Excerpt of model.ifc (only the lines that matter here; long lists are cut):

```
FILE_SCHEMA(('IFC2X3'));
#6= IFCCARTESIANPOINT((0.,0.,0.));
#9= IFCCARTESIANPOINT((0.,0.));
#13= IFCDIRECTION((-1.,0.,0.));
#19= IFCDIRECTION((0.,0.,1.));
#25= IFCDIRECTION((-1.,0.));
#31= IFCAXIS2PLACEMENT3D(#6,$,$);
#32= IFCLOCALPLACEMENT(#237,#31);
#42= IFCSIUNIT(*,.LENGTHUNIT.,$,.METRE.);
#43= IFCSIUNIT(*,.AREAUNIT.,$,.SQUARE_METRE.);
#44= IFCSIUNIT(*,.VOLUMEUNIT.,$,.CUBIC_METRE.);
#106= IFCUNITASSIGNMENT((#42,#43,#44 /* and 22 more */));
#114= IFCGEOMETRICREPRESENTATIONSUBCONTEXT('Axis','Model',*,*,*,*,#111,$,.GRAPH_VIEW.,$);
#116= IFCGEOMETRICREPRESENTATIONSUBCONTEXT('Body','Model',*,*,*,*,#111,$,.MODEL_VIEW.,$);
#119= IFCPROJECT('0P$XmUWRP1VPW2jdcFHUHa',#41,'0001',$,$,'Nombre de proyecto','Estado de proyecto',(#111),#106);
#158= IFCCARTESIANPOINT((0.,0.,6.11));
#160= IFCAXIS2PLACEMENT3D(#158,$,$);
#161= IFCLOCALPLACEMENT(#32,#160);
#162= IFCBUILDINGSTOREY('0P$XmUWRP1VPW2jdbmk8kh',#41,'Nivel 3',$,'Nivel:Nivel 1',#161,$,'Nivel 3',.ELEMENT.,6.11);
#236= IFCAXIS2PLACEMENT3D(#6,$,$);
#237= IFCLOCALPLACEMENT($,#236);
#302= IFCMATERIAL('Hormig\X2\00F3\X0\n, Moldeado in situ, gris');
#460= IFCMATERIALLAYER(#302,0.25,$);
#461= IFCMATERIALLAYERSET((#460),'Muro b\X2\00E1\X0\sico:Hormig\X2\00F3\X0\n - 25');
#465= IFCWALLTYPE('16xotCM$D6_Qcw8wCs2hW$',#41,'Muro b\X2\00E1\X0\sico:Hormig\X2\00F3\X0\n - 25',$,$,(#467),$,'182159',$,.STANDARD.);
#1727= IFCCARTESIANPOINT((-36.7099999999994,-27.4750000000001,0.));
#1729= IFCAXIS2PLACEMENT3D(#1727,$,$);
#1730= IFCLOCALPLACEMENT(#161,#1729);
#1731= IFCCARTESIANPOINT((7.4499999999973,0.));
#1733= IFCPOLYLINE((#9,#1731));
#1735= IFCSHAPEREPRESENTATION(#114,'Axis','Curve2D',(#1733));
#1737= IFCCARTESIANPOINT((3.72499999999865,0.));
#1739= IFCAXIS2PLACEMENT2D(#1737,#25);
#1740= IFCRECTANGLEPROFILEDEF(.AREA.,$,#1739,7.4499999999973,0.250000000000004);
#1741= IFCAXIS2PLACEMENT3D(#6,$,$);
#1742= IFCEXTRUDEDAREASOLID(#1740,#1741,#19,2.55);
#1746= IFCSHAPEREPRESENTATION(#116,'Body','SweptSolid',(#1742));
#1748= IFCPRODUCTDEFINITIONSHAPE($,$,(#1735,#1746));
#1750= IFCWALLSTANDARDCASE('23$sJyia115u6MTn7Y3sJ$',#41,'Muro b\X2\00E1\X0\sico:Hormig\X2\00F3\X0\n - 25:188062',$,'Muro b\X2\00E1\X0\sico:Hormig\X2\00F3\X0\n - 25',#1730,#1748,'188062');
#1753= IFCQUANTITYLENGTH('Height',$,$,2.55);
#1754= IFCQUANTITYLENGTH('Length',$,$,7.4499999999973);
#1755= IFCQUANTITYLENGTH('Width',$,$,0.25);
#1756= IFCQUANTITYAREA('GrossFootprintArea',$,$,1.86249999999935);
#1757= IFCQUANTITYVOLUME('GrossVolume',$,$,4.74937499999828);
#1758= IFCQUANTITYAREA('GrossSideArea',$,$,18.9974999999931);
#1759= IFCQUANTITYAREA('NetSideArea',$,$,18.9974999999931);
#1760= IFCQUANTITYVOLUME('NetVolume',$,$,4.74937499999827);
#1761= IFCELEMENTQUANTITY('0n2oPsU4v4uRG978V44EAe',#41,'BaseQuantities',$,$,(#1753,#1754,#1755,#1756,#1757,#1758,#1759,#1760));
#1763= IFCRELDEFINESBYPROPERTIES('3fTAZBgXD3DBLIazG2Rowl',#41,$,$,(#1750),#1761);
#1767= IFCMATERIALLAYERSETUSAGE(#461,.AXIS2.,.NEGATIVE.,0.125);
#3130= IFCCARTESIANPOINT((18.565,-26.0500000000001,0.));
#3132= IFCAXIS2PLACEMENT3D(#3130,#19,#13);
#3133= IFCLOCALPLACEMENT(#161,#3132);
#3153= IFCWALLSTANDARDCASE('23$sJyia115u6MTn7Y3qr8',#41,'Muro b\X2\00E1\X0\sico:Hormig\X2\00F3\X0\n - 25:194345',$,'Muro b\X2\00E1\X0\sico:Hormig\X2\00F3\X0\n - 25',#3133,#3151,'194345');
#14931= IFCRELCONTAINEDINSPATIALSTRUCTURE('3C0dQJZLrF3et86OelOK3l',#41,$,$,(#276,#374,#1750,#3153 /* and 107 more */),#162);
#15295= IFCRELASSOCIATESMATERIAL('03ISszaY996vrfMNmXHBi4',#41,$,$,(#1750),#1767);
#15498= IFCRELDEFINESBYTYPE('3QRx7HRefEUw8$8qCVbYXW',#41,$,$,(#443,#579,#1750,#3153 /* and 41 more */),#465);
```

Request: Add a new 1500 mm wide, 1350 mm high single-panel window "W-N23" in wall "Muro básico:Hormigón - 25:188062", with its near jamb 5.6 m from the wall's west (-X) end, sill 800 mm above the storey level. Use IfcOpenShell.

```python
import numpy as np
import ifcopenshell
import ifcopenshell.api.feature
import ifcopenshell.api.geometry
import ifcopenshell.api.pset
import ifcopenshell.api.root
import ifcopenshell.api.spatial
import ifcopenshell.api.type
import ifcopenshell.geom
import ifcopenshell.util.element
import ifcopenshell.util.placement
import ifcopenshell.util.representation
import ifcopenshell.util.shape
import ifcopenshell.util.unit

model = ifcopenshell.open("model.ifc")
unit_scale = ifcopenshell.util.unit.calculate_unit_scale(model)
area_scale = ifcopenshell.util.unit.calculate_unit_scale(model, "AREAUNIT")
volume_scale = ifcopenshell.util.unit.calculate_unit_scale(model, "VOLUMEUNIT")
settings = ifcopenshell.geom.settings()


def volume(element):
    """Net volume in cubic metres, openings subtracted."""
    shape = ifcopenshell.geom.create_shape(settings, element)
    return ifcopenshell.util.shape.get_volume(shape.geometry)


wall = model.by_guid("23$sJyia115u6MTn7Y3sJ$")
storey = ifcopenshell.util.element.get_container(wall, ifc_class="IfcBuildingStorey")
context = ifcopenshell.util.representation.get_context(model, "Model", "Body", "MODEL_VIEW")
before = volume(wall)

width, height, from_end, sill = 1.5, 1.35, 5.6, 0.8  # metres

# The wall runs along its own X axis, and the end named is its -X end.
wall_shape = ifcopenshell.geom.create_shape(settings, wall)
x, y, z = ifcopenshell.util.shape.get_vertices(wall_shape.geometry).T
start = x.min() + from_end
face, thickness = float(y.min()), float(y.max() - y.min())
wall_matrix = ifcopenshell.util.placement.get_local_placement(wall.ObjectPlacement)
level = ifcopenshell.util.placement.get_local_placement(storey.ObjectPlacement)[2, 3]


def in_wall(x, y):
    """Placement at x, y metres in the wall's axes, at sill height."""
    matrix = wall_matrix.copy()
    matrix[:, 3] = wall_matrix @ np.array([x / unit_scale, y / unit_scale, 0.0, 1.0])
    matrix[2, 3] = level + sill / unit_scale
    return matrix


# Opening: a box that overshoots both wall faces by 50 mm.
opening = ifcopenshell.api.root.create_entity(model, ifc_class="IfcOpeningElement")
box = ifcopenshell.api.geometry.add_wall_representation(
    model, context=context, length=width, height=height, thickness=thickness + 0.1
)
ifcopenshell.api.geometry.assign_representation(model, product=opening, representation=box)
ifcopenshell.api.geometry.edit_object_placement(model, product=opening, matrix=in_wall(start, face - 0.05), is_si=False)
ifcopenshell.api.feature.add_feature(model, feature=opening, element=wall)

window = ifcopenshell.api.root.create_entity(model, ifc_class="IfcWindow", name="W-N23")
window.OverallWidth, window.OverallHeight = width / unit_scale, height / unit_scale
body = ifcopenshell.api.geometry.add_window_representation(
    model,
    context=context,
    overall_width=window.OverallWidth,
    overall_height=window.OverallHeight,
    partition_type="SINGLE_PANEL",
)
ifcopenshell.api.geometry.assign_representation(model, product=window, representation=body)
ifcopenshell.api.spatial.assign_container(model, products=[window], relating_structure=storey)
fills = ifcopenshell.api.feature.add_filling(model, opening=opening, element=window)
fills.OwnerHistory = window.OwnerHistory  # required in IFC2X3

# IFC2X3 keeps the operation on the window style.
style = ifcopenshell.api.root.create_entity(model, ifc_class="IfcWindowStyle", name="W-N23")
style.OperationType, style.ConstructionType = "SINGLE_PANEL", "NOTDEFINED"
style.ParameterTakesPrecedence = style.Sizeable = False
ifcopenshell.api.type.assign_type(model, related_objects=[window], relating_type=style)

# Centre the window in the wall's thickness.
ifcopenshell.api.geometry.edit_object_placement(model, product=window, matrix=in_wall(start, face), is_si=False)
window_shape = ifcopenshell.geom.create_shape(settings, window)
depth = ifcopenshell.util.shape.get_vertices(window_shape.geometry)[:, 1]
offset = face + thickness / 2 - (depth.min() + depth.max()) / 2
ifcopenshell.api.geometry.edit_object_placement(model, product=window, matrix=in_wall(start, offset), is_si=False)

after = volume(wall)

# Update the wall's stored quantities.
qto = model.by_id(ifcopenshell.util.element.get_pset(wall, "BaseQuantities", should_inherit=False)["id"])
ifcopenshell.api.pset.edit_qto(model, qto=qto, properties={
    "NetSideArea": after / thickness / area_scale,
    "NetVolume": after / volume_scale,
})

print(f"wall volume {before:.3f} -> {after:.3f} m3")

model.write("model_rev.ifc")
```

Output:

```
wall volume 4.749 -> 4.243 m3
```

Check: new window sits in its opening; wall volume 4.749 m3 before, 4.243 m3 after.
